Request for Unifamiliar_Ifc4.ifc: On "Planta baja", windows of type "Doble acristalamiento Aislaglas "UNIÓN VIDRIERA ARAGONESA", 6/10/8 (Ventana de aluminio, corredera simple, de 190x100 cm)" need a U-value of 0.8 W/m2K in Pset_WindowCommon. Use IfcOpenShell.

First a look at what the model holds.

```python
import ifcopenshell
import ifcopenshell.util.element

model = ifcopenshell.open("Unifamiliar_Ifc4.ifc")
print(model.schema)
storey = next(s for s in model.by_type("IfcBuildingStorey") if s.Name == "Planta baja")
windows = [e for e in ifcopenshell.util.element.get_decomposition(storey) if e.is_a("IfcWindow")]
seen = {}
for e in windows:
    element_type = ifcopenshell.util.element.get_type(e)
    key = (element_type.Name if element_type != e and element_type else None, ifcopenshell.util.element.get_pset(e, "Pset_WindowCommon", "ThermalTransmittance"))
    seen[key] = seen.get(key, 0) + 1
for (name, value), count in sorted(seen.items(), key=str):
    print(count, "x", name, "|", value)
```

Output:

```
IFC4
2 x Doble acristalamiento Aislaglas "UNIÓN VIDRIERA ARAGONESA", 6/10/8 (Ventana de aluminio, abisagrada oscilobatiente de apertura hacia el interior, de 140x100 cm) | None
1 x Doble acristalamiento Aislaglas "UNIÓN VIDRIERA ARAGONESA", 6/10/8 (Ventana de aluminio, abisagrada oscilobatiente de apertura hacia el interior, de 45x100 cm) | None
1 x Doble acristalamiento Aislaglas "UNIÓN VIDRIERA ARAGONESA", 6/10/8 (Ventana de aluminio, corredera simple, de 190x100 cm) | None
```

```python
import ifcopenshell
import ifcopenshell.api.pset
import ifcopenshell.util.element

model = ifcopenshell.open("Unifamiliar_Ifc4.ifc")

storey = next(s for s in model.by_type("IfcBuildingStorey") if s.Name == "Planta baja")
windows = [e for e in ifcopenshell.util.element.get_decomposition(storey) if e.is_a("IfcWindow")]

count = 0
for e in windows:
    element_type = ifcopenshell.util.element.get_type(e)
    if element_type in (None, e) or element_type.Name != 'Doble acristalamiento Aislaglas "UNIÓN VIDRIERA ARAGONESA", 6/10/8 (Ventana de aluminio, corredera simple, de 190x100 cm)':
        continue
    # add_pset returns the element's existing set when there is one.
    pset = ifcopenshell.api.pset.add_pset(model, product=e, name="Pset_WindowCommon")
    ifcopenshell.api.pset.edit_pset(model, pset=pset, properties={"ThermalTransmittance": 0.8})
    count += 1

print(count, "windows updated")

model.write("Unifamiliar_Ifc4-out.ifc")
```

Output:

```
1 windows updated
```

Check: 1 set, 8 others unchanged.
